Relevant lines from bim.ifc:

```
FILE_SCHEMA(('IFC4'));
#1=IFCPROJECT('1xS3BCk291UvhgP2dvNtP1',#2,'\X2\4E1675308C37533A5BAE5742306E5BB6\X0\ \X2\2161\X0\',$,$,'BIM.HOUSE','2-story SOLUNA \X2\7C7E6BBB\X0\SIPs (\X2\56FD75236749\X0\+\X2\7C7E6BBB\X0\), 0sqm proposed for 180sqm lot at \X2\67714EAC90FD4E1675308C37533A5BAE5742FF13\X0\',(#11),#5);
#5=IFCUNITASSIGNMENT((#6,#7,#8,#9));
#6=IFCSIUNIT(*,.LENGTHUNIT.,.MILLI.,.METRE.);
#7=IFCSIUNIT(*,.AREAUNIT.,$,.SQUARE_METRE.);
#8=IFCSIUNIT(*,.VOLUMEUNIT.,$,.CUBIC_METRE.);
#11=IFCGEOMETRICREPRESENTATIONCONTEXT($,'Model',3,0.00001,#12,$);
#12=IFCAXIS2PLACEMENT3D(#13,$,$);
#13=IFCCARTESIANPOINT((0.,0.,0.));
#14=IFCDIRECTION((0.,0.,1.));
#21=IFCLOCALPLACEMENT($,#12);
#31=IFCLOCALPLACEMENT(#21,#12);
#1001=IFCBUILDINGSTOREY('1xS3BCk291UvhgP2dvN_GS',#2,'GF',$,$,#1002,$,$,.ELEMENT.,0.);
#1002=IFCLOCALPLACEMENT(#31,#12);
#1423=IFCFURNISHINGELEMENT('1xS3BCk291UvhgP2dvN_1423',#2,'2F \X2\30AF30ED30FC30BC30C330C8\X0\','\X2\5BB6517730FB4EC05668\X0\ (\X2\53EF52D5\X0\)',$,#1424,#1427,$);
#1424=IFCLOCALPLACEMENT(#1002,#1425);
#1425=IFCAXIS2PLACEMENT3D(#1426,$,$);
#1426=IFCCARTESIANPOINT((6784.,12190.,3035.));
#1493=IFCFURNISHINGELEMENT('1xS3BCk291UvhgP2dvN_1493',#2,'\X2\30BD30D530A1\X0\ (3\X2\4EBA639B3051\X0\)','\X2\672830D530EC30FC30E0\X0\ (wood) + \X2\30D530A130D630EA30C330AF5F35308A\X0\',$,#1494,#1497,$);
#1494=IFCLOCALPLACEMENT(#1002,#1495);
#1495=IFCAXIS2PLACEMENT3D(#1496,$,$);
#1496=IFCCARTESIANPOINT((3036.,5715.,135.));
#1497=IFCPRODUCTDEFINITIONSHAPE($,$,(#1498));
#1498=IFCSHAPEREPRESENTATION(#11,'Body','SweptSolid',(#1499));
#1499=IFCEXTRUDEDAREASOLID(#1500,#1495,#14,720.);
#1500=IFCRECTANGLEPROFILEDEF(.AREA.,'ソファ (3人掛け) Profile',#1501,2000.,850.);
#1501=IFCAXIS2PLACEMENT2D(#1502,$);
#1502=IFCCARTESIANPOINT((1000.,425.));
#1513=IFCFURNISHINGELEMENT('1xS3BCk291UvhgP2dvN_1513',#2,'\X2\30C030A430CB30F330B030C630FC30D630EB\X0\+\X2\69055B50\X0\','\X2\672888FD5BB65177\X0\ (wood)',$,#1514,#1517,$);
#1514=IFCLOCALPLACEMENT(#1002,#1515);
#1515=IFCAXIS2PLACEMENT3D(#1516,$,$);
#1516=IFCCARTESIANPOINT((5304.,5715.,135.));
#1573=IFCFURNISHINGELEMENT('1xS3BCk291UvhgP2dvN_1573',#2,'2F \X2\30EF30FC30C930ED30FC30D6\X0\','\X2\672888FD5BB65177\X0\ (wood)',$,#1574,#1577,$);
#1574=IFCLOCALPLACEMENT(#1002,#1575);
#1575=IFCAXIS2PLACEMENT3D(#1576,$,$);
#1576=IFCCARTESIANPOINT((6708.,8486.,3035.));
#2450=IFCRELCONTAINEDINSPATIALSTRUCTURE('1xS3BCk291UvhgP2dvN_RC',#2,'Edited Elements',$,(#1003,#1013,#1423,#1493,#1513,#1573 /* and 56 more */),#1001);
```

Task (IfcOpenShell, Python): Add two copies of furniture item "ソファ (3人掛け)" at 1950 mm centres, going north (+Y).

```python
import numpy as np
import ifcopenshell
import ifcopenshell.api.geometry
import ifcopenshell.api.root
import ifcopenshell.util.element
import ifcopenshell.util.placement

model = ifcopenshell.open("bim.ifc")


def reuse_history(source, copy):
    """copy_class also copies each property set's owner history, people and application; keep the originals."""
    for rel in copy.IsDefinedBy:
        if rel.is_a("IfcRelDefinesByProperties") and (history := rel.RelatingPropertyDefinition.OwnerHistory):
            rel.RelatingPropertyDefinition.OwnerHistory = source.OwnerHistory
            ifcopenshell.util.element.remove_deep2(model, history)


source = model.by_guid("1xS3BCk291UvhgP2dvN_1493")
base = ifcopenshell.util.placement.get_local_placement(source.ObjectPlacement)
step = np.array([0.0, 1.0, 0.0]) * 1950.0

for i in range(1, 3):
    copy = ifcopenshell.api.root.copy_class(model, product=source)
    copy.Representation = ifcopenshell.util.element.copy_deep(
        model, source.Representation, exclude=["IfcGeometricRepresentationContext", "IfcRepresentationMap"]
    )
    reuse_history(source, copy)
    matrix = base.copy()
    matrix[:3, 3] += i * step
    print("added at", matrix[:3, 3].round(3) + 0.0)
    ifcopenshell.api.geometry.edit_object_placement(model, product=copy, matrix=matrix, is_si=False)

model.write("bim_v2.ifc")
```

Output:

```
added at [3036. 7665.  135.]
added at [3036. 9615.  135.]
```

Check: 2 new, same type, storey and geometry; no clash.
